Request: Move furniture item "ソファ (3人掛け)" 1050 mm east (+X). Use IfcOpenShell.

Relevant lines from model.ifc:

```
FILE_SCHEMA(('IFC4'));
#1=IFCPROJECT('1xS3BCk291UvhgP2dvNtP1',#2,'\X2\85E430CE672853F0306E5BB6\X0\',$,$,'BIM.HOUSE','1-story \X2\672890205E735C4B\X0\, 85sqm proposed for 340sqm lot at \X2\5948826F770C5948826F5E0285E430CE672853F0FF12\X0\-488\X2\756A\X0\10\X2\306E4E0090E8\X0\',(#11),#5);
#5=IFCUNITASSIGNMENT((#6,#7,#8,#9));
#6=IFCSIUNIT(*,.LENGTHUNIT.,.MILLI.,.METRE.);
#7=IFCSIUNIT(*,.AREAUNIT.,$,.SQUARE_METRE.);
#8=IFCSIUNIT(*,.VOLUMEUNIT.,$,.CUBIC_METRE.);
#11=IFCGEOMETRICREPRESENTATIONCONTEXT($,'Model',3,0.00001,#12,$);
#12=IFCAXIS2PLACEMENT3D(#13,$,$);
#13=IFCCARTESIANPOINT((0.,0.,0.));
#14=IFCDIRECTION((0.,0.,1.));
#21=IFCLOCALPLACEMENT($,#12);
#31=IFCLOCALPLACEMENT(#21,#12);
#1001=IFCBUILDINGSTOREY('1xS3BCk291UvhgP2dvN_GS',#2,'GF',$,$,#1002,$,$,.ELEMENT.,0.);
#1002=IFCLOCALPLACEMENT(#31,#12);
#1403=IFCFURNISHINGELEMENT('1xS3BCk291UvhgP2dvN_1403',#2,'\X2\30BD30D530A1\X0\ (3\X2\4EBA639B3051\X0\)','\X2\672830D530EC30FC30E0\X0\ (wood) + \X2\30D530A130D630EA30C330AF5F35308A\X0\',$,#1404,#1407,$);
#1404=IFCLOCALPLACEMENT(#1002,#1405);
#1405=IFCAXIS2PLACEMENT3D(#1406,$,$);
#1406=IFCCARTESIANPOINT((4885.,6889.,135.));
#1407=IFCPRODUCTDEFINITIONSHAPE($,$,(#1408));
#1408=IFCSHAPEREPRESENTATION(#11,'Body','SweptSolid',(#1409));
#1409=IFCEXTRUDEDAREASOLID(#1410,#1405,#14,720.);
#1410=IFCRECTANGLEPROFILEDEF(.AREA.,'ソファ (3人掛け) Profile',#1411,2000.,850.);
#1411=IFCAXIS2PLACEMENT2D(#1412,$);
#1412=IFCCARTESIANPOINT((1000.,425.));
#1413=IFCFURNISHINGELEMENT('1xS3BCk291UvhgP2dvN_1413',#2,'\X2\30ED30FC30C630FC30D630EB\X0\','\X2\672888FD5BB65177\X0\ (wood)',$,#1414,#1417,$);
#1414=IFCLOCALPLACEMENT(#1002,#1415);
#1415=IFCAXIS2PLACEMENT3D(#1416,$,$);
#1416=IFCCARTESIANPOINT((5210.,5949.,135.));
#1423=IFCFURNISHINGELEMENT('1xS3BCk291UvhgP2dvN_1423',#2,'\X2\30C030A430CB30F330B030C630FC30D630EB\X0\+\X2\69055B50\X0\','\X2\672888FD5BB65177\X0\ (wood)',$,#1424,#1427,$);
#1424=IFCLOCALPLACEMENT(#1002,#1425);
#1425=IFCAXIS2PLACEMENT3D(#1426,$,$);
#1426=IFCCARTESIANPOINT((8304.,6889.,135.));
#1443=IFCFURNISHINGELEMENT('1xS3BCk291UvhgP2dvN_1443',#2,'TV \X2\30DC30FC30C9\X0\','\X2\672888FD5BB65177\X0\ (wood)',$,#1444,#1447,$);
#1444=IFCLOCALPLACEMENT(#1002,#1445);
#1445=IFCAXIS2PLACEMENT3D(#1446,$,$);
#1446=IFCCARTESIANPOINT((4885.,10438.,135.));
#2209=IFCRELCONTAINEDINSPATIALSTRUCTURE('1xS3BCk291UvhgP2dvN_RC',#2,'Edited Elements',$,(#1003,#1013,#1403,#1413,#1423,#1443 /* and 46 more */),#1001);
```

```python
import ifcopenshell
import ifcopenshell.api.geometry
import ifcopenshell.util.placement
import ifcopenshell.util.unit

model = ifcopenshell.open("model.ifc")
unit_scale = ifcopenshell.util.unit.calculate_unit_scale(model)

item = model.by_guid("1xS3BCk291UvhgP2dvN_1403")
matrix = ifcopenshell.util.placement.get_local_placement(item.ObjectPlacement)
matrix[0, 3] += 1.05 / unit_scale
ifcopenshell.api.geometry.edit_object_placement(model, product=item, matrix=matrix, is_si=False)

print(ifcopenshell.util.placement.get_local_placement(item.ObjectPlacement).round(3) + 0.0)

model.write("model_edited.ifc")
```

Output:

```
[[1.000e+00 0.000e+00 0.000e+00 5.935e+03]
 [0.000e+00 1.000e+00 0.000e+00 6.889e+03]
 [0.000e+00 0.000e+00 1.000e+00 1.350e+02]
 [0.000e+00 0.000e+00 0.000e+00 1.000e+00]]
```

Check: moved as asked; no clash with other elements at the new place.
